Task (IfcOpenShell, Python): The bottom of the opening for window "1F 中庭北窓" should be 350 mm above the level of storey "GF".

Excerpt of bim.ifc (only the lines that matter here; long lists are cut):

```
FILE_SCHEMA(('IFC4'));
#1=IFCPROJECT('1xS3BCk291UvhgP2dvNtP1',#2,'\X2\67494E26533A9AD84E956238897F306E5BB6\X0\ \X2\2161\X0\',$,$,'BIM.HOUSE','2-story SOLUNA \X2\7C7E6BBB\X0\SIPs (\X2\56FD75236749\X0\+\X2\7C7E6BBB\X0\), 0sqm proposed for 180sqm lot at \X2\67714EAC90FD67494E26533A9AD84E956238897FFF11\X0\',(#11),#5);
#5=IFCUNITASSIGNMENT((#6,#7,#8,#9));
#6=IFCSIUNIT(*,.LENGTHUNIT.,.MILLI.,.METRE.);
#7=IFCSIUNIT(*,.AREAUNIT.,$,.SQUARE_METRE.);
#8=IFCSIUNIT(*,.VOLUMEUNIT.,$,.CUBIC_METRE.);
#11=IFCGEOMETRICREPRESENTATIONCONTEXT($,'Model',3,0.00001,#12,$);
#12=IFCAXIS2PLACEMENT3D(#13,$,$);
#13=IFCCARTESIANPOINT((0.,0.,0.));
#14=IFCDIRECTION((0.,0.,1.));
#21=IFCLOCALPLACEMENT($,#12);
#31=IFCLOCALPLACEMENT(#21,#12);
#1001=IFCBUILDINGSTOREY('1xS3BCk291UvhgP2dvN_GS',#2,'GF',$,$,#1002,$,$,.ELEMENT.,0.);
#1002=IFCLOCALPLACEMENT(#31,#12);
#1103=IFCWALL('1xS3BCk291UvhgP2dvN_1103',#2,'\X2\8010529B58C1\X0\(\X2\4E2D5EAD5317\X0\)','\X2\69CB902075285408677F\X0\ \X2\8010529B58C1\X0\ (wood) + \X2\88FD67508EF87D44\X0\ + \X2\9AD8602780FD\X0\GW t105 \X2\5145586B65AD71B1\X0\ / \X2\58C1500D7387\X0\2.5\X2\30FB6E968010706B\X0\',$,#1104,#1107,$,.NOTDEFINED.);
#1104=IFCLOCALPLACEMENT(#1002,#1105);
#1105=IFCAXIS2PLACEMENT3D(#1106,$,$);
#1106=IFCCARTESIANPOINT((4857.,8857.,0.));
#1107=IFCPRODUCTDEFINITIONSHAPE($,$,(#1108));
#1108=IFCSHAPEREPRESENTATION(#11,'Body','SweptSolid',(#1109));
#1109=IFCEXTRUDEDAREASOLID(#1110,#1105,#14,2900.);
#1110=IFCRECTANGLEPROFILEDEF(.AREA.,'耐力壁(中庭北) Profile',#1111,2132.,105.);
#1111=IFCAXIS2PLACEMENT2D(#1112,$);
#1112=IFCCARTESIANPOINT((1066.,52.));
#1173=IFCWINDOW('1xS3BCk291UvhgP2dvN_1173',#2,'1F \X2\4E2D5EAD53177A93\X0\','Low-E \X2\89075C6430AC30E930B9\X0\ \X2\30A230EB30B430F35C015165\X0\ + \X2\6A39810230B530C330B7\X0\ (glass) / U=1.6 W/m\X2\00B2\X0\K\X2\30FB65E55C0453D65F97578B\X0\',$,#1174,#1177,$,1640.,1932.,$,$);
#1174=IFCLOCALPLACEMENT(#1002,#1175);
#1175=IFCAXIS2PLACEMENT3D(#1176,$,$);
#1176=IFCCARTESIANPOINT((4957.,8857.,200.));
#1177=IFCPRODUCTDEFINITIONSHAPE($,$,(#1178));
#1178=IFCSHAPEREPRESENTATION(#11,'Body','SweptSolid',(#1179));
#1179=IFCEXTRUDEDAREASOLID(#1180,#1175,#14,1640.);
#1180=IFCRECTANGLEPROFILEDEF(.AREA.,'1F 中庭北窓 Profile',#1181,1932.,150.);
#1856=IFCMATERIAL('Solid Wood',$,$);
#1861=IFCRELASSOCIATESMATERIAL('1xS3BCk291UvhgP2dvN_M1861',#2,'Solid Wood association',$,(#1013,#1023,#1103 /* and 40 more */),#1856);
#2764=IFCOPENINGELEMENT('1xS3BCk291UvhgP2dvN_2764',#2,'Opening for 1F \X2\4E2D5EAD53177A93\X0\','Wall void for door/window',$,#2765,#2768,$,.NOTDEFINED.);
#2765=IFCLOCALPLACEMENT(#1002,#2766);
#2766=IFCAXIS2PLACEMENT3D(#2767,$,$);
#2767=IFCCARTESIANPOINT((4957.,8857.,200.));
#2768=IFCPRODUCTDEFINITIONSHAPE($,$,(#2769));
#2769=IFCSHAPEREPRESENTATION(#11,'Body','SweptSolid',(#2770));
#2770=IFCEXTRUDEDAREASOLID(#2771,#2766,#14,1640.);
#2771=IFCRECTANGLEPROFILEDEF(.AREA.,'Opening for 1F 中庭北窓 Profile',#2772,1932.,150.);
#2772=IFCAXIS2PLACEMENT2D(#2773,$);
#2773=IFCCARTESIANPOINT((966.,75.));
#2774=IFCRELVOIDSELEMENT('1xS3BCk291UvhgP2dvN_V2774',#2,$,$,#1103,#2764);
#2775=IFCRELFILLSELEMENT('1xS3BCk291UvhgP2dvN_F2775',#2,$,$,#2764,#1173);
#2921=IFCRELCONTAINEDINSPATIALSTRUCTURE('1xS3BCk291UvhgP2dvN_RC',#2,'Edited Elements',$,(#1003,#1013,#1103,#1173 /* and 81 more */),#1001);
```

```python
import numpy as np
import ifcopenshell
import ifcopenshell.api.geometry
import ifcopenshell.geom
import ifcopenshell.util.element
import ifcopenshell.util.placement
import ifcopenshell.util.shape
import ifcopenshell.util.unit

model = ifcopenshell.open("bim.ifc")
unit_scale = ifcopenshell.util.unit.calculate_unit_scale(model)

window = model.by_guid("1xS3BCk291UvhgP2dvN_1173")
opening = window.FillsVoids[0].RelatingOpeningElement
storey = ifcopenshell.util.element.get_container(window, ifc_class="IfcBuildingStorey")
level = ifcopenshell.util.placement.get_local_placement(storey.ObjectPlacement)[2, 3]

# The opening's origin need not be at the sill, so measure its lowest point.
shape = ifcopenshell.geom.create_shape(ifcopenshell.geom.settings(), opening)
bottom = ifcopenshell.util.shape.get_shape_bottom_elevation(shape, shape.geometry) / unit_scale
dz = level + 350.0 - bottom

shift = np.array([0.0, 0.0, dz])
# The window is not placed relative to its opening, so move both.
for product in (opening, window):
    matrix = ifcopenshell.util.placement.get_local_placement(product.ObjectPlacement)
    matrix[:3, 3] += shift
    ifcopenshell.api.geometry.edit_object_placement(model, product=product, matrix=matrix, is_si=False)

print(f"moved by {dz * unit_scale:+.3f} m")

model.write("bim_updated.ifc")
```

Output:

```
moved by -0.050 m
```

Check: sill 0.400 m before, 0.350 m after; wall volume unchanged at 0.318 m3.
